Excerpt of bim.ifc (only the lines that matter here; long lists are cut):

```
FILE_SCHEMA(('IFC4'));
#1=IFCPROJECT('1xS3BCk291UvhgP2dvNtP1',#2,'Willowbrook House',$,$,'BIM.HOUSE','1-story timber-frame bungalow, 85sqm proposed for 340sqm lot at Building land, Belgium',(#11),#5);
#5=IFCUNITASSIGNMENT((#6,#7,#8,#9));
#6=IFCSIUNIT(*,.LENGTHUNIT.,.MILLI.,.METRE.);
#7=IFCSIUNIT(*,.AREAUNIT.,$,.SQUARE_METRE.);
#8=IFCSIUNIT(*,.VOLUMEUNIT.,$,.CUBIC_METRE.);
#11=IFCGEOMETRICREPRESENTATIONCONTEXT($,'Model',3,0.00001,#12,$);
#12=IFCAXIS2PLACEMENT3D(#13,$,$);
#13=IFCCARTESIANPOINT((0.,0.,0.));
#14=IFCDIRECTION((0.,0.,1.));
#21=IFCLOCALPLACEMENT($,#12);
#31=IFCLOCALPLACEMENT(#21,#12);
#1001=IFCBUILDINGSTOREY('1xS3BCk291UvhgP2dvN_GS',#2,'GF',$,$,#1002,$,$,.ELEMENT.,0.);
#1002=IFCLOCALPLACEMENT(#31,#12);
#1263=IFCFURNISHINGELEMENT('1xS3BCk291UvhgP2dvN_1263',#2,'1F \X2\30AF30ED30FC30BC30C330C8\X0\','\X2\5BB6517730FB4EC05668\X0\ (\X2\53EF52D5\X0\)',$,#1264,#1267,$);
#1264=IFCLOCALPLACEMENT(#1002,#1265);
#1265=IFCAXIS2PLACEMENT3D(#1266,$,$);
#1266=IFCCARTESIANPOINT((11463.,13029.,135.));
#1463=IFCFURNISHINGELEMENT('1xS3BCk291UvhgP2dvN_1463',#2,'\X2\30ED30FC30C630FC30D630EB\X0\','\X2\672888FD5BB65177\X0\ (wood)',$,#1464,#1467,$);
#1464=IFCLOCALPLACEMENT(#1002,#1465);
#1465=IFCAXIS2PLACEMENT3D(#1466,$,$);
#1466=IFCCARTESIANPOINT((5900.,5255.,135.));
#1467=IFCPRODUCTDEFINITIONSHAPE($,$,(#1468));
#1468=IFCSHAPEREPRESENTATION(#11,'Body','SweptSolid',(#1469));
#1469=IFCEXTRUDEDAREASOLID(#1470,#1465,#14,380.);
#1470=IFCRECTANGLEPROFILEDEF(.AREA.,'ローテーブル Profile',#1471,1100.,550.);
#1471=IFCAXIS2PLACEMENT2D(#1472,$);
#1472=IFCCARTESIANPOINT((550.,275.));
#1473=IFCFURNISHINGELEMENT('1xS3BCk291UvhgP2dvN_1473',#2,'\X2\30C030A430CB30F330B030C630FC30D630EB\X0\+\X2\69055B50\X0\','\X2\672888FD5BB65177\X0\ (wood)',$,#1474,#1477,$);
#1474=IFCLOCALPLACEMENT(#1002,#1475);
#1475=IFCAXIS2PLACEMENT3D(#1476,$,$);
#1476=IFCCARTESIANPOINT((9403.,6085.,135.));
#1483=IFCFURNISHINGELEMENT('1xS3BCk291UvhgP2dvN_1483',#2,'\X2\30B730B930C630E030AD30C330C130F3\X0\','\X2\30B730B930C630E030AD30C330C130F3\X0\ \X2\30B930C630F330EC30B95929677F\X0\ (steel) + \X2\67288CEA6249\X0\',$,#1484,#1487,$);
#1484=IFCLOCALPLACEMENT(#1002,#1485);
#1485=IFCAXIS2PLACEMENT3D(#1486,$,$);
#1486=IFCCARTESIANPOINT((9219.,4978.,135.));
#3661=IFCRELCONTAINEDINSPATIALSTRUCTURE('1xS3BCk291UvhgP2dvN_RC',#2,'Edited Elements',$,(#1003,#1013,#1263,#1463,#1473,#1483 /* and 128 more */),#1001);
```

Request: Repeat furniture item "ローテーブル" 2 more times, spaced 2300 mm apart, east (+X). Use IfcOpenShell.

```python
import numpy as np
import ifcopenshell
import ifcopenshell.api.geometry
import ifcopenshell.api.root
import ifcopenshell.util.element
import ifcopenshell.util.placement

model = ifcopenshell.open("bim.ifc")


def reuse_history(source, copy):
    """copy_class also copies each property set's owner history, people and application; keep the originals."""
    for rel in copy.IsDefinedBy:
        if rel.is_a("IfcRelDefinesByProperties") and (history := rel.RelatingPropertyDefinition.OwnerHistory):
            rel.RelatingPropertyDefinition.OwnerHistory = source.OwnerHistory
            ifcopenshell.util.element.remove_deep2(model, history)


source = model.by_id(1463)
base = ifcopenshell.util.placement.get_local_placement(source.ObjectPlacement)
step = np.array([1.0, 0.0, 0.0]) * 2300.0

for i in range(1, 3):
    copy = ifcopenshell.api.root.copy_class(model, product=source)
    copy.Representation = ifcopenshell.util.element.copy_deep(
        model, source.Representation, exclude=["IfcGeometricRepresentationContext", "IfcRepresentationMap"]
    )
    reuse_history(source, copy)
    matrix = base.copy()
    matrix[:3, 3] += i * step
    print("added at", matrix[:3, 3].round(3) + 0.0)
    ifcopenshell.api.geometry.edit_object_placement(model, product=copy, matrix=matrix, is_si=False)

model.write("bim_rev.ifc")
```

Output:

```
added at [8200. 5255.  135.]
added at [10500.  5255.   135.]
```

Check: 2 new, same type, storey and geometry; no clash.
